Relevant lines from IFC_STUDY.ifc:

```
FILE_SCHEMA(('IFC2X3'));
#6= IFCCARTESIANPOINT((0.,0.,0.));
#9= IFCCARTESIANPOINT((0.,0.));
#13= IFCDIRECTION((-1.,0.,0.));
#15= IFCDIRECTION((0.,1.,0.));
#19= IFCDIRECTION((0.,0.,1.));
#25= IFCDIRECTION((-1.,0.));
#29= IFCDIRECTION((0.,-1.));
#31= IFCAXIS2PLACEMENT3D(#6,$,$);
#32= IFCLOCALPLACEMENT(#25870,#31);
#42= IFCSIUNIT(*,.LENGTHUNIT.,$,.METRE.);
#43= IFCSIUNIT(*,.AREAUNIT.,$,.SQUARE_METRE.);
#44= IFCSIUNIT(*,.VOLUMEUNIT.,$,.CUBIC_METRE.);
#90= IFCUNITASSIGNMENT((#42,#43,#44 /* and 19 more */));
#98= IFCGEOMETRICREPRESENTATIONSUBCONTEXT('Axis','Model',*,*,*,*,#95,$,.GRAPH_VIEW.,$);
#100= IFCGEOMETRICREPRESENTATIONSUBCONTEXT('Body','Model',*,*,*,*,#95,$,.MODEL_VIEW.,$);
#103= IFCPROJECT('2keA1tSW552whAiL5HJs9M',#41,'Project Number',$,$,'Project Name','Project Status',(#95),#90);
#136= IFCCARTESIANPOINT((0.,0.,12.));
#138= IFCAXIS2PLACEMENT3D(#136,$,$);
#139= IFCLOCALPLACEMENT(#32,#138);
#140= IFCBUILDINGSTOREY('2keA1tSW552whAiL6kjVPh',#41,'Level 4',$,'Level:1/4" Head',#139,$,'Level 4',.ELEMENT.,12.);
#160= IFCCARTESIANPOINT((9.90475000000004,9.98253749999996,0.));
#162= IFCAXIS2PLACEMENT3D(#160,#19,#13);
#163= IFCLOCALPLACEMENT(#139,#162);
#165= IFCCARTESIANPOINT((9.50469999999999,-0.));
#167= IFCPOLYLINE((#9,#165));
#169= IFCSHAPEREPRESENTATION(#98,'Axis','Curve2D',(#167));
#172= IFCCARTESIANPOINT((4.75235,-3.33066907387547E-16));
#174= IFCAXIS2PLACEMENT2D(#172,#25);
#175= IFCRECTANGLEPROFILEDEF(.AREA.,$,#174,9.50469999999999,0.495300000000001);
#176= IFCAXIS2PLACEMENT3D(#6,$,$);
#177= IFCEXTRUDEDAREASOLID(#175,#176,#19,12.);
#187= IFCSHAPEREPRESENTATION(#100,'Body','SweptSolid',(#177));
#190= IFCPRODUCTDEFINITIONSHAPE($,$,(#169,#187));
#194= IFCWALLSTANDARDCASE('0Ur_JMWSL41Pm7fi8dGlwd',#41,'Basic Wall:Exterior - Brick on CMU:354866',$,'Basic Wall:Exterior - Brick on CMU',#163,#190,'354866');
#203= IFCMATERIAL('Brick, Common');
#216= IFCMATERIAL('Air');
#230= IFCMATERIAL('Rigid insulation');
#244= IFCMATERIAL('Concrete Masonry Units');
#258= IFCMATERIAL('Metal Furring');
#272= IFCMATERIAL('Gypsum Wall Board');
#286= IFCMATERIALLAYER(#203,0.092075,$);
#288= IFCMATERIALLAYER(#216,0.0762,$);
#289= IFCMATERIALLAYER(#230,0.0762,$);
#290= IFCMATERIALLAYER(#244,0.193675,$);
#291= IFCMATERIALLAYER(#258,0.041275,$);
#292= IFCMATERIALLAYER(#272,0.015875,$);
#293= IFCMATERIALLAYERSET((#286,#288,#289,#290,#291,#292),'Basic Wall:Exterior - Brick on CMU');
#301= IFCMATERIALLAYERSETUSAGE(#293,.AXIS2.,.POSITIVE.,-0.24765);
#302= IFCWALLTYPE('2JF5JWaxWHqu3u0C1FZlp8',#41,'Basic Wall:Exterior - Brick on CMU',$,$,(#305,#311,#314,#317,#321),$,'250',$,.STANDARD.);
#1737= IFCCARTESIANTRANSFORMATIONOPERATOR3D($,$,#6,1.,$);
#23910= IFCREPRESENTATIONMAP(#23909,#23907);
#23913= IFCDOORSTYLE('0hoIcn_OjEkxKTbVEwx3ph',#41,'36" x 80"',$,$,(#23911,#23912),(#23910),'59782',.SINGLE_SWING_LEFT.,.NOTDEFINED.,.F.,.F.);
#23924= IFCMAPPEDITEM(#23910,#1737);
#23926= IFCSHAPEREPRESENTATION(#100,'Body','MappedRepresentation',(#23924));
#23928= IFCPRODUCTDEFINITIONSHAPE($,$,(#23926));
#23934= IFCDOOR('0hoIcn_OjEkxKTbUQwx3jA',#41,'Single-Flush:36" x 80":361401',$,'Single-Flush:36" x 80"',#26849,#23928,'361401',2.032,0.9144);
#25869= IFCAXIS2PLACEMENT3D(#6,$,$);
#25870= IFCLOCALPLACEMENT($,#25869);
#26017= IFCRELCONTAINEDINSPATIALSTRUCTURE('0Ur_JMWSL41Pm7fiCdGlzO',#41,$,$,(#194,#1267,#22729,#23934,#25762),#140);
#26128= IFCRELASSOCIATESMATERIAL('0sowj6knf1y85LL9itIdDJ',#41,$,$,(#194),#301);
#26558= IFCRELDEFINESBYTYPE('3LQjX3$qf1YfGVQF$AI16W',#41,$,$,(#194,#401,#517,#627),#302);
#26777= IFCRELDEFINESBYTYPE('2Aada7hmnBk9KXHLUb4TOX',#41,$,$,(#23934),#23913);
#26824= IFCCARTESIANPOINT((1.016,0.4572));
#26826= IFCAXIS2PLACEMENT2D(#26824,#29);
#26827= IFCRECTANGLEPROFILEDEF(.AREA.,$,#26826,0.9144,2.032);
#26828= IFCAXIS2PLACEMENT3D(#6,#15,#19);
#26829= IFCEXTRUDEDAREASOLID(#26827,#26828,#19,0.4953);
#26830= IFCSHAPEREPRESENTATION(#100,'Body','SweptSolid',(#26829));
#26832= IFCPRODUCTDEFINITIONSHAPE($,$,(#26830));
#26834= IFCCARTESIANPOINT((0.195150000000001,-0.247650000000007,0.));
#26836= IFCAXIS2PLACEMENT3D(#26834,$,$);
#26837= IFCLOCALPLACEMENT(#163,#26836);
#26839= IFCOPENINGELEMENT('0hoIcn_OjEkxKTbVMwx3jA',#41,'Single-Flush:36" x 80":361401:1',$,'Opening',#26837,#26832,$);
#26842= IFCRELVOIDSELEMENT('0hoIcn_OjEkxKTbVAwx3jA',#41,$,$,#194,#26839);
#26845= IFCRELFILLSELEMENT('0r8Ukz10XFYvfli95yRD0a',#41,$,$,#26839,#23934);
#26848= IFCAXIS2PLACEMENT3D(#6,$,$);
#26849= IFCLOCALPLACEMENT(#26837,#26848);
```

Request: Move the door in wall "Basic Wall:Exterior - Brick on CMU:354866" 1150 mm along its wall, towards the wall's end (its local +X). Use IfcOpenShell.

```python
import ifcopenshell
import ifcopenshell.api.geometry
import ifcopenshell.util.placement
import ifcopenshell.util.unit

model = ifcopenshell.open("IFC_STUDY.ifc")
unit_scale = ifcopenshell.util.unit.calculate_unit_scale(model)

door = model.by_id(23934)
opening = door.FillsVoids[0].RelatingOpeningElement
wall = opening.VoidsElements[0].RelatingBuildingElement

wall_matrix = ifcopenshell.util.placement.get_local_placement(wall.ObjectPlacement)
shift = wall_matrix[:3, 0] * 1.15 / unit_scale
before = ifcopenshell.util.placement.get_local_placement(door.ObjectPlacement)[:3, 3].copy()

# The door is placed relative to its opening, so it follows when the opening moves.
matrix = ifcopenshell.util.placement.get_local_placement(opening.ObjectPlacement)
matrix[:3, 3] += shift
ifcopenshell.api.geometry.edit_object_placement(
    model, product=opening, matrix=matrix, is_si=False, should_transform_children=True
)

after = ifcopenshell.util.placement.get_local_placement(door.ObjectPlacement)[:3, 3]
print("door moved by", (after - before).round(3) + 0.0)

model.write("IFC_STUDY-out.ifc")
```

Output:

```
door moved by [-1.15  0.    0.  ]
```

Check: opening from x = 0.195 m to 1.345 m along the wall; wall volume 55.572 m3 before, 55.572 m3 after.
